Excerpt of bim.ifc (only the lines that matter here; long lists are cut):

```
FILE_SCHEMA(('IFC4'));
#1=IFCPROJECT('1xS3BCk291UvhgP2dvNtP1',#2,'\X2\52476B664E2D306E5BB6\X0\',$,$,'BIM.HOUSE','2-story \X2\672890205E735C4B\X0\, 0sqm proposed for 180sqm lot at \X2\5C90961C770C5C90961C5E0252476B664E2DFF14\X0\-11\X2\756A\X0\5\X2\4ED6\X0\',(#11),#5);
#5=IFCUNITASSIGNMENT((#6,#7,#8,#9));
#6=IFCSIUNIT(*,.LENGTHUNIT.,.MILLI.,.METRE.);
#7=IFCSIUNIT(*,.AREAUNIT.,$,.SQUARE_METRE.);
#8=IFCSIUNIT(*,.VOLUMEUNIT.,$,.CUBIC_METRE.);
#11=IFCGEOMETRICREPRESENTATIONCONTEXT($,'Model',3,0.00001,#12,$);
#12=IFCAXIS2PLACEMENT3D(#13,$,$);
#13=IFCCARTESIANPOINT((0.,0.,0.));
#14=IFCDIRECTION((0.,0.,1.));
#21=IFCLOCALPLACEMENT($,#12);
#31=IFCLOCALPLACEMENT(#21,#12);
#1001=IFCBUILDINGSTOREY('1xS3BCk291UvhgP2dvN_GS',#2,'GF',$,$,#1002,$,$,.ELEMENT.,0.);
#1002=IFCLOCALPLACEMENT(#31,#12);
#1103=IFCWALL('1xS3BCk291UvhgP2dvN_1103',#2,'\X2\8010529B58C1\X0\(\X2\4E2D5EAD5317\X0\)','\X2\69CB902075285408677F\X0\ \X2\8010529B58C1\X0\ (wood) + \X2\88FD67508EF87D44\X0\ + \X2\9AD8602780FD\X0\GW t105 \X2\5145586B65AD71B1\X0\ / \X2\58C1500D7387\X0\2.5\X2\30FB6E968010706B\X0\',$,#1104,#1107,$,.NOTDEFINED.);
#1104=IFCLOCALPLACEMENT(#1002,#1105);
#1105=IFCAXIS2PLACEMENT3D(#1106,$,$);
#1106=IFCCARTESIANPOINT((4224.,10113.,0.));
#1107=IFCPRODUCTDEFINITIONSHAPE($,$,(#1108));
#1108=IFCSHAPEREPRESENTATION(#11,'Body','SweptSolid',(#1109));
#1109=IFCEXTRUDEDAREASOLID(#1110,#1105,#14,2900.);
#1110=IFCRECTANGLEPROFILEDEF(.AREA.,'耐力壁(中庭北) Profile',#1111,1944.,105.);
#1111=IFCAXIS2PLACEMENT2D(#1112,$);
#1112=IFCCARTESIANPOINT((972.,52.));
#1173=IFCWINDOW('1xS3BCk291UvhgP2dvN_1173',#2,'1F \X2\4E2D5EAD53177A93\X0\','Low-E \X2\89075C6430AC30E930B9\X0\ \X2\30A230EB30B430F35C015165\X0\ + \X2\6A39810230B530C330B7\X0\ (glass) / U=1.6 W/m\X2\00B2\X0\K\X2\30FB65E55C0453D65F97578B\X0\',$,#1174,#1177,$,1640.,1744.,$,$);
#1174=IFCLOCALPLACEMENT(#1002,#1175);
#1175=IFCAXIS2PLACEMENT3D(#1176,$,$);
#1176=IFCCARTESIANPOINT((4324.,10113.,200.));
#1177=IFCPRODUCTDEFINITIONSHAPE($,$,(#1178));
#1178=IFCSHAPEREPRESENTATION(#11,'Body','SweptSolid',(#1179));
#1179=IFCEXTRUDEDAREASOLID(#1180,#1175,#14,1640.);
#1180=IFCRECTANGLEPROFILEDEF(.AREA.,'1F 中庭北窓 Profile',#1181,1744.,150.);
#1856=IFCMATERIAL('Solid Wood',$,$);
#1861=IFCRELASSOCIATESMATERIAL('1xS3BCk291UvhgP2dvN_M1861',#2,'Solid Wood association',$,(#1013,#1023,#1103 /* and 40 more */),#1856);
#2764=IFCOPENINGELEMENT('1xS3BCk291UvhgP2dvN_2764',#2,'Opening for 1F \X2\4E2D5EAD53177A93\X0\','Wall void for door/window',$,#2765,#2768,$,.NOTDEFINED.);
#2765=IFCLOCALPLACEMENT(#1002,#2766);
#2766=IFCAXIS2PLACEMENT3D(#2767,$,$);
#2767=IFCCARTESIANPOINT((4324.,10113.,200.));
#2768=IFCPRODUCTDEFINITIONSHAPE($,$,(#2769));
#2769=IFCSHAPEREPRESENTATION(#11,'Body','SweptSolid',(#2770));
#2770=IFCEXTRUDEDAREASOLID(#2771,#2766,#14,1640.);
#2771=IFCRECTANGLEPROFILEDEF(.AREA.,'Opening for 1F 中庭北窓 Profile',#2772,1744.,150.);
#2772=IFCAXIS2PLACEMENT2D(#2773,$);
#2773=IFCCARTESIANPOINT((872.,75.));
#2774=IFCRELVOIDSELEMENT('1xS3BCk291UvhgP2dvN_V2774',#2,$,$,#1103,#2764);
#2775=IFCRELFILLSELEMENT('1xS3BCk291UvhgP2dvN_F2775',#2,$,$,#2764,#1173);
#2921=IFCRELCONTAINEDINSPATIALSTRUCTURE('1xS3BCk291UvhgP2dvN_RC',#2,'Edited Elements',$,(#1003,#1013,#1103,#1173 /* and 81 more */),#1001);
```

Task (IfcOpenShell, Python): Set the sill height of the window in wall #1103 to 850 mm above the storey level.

```python
import numpy as np
import ifcopenshell
import ifcopenshell.api.geometry
import ifcopenshell.geom
import ifcopenshell.util.element
import ifcopenshell.util.placement
import ifcopenshell.util.shape
import ifcopenshell.util.unit

model = ifcopenshell.open("bim.ifc")
unit_scale = ifcopenshell.util.unit.calculate_unit_scale(model)

window = model.by_guid("1xS3BCk291UvhgP2dvN_1173")
opening = window.FillsVoids[0].RelatingOpeningElement
storey = ifcopenshell.util.element.get_container(window, ifc_class="IfcBuildingStorey")
level = ifcopenshell.util.placement.get_local_placement(storey.ObjectPlacement)[2, 3]

# The opening's origin need not be at the sill, so measure its lowest point.
shape = ifcopenshell.geom.create_shape(ifcopenshell.geom.settings(), opening)
bottom = ifcopenshell.util.shape.get_shape_bottom_elevation(shape, shape.geometry) / unit_scale
dz = level + 0.85 / unit_scale - bottom

shift = np.array([0.0, 0.0, dz])
# The window is not placed relative to its opening, so move both.
for product in (opening, window):
    matrix = ifcopenshell.util.placement.get_local_placement(product.ObjectPlacement)
    matrix[:3, 3] += shift
    ifcopenshell.api.geometry.edit_object_placement(model, product=product, matrix=matrix, is_si=False)

print(f"moved by {dz * unit_scale:+.3f} m")

model.write("bim_rev.ifc")
```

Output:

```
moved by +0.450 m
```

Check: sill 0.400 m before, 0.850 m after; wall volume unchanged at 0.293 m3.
